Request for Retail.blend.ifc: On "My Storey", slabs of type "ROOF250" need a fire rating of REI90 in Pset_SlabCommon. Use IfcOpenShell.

First a look at what the model holds.

```python
import ifcopenshell
import ifcopenshell.util.element

model = ifcopenshell.open("Retail.blend.ifc")
print(model.schema)
storey = next(s for s in model.by_type("IfcBuildingStorey") if s.Name == "My Storey")
slabs = [e for e in ifcopenshell.util.element.get_decomposition(storey) if e.is_a("IfcSlab")]
seen = {}
for e in slabs:
    element_type = ifcopenshell.util.element.get_type(e)
    key = (element_type.Name if element_type != e and element_type else None, ifcopenshell.util.element.get_pset(e, "Pset_SlabCommon", "FireRating"))
    seen[key] = seen.get(key, 0) + 1
for (name, value), count in sorted(seen.items(), key=str):
    print(count, "x", name, "|", value)
```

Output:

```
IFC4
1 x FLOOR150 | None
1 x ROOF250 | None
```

```python
import ifcopenshell
import ifcopenshell.api.pset
import ifcopenshell.util.element

model = ifcopenshell.open("Retail.blend.ifc")

storey = next(s for s in model.by_type("IfcBuildingStorey") if s.Name == "My Storey")
slabs = [e for e in ifcopenshell.util.element.get_decomposition(storey) if e.is_a("IfcSlab")]

count = 0
for e in slabs:
    element_type = ifcopenshell.util.element.get_type(e)
    if element_type in (None, e) or element_type.Name != "ROOF250":
        continue
    # add_pset returns the element's existing set when there is one.
    pset = ifcopenshell.api.pset.add_pset(model, product=e, name="Pset_SlabCommon")
    ifcopenshell.api.pset.edit_pset(model, pset=pset, properties={"FireRating": "REI90"})
    count += 1

print(count, "slabs updated")

model.write("Retail.blend_rev.ifc")
```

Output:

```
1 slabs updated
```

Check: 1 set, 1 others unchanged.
